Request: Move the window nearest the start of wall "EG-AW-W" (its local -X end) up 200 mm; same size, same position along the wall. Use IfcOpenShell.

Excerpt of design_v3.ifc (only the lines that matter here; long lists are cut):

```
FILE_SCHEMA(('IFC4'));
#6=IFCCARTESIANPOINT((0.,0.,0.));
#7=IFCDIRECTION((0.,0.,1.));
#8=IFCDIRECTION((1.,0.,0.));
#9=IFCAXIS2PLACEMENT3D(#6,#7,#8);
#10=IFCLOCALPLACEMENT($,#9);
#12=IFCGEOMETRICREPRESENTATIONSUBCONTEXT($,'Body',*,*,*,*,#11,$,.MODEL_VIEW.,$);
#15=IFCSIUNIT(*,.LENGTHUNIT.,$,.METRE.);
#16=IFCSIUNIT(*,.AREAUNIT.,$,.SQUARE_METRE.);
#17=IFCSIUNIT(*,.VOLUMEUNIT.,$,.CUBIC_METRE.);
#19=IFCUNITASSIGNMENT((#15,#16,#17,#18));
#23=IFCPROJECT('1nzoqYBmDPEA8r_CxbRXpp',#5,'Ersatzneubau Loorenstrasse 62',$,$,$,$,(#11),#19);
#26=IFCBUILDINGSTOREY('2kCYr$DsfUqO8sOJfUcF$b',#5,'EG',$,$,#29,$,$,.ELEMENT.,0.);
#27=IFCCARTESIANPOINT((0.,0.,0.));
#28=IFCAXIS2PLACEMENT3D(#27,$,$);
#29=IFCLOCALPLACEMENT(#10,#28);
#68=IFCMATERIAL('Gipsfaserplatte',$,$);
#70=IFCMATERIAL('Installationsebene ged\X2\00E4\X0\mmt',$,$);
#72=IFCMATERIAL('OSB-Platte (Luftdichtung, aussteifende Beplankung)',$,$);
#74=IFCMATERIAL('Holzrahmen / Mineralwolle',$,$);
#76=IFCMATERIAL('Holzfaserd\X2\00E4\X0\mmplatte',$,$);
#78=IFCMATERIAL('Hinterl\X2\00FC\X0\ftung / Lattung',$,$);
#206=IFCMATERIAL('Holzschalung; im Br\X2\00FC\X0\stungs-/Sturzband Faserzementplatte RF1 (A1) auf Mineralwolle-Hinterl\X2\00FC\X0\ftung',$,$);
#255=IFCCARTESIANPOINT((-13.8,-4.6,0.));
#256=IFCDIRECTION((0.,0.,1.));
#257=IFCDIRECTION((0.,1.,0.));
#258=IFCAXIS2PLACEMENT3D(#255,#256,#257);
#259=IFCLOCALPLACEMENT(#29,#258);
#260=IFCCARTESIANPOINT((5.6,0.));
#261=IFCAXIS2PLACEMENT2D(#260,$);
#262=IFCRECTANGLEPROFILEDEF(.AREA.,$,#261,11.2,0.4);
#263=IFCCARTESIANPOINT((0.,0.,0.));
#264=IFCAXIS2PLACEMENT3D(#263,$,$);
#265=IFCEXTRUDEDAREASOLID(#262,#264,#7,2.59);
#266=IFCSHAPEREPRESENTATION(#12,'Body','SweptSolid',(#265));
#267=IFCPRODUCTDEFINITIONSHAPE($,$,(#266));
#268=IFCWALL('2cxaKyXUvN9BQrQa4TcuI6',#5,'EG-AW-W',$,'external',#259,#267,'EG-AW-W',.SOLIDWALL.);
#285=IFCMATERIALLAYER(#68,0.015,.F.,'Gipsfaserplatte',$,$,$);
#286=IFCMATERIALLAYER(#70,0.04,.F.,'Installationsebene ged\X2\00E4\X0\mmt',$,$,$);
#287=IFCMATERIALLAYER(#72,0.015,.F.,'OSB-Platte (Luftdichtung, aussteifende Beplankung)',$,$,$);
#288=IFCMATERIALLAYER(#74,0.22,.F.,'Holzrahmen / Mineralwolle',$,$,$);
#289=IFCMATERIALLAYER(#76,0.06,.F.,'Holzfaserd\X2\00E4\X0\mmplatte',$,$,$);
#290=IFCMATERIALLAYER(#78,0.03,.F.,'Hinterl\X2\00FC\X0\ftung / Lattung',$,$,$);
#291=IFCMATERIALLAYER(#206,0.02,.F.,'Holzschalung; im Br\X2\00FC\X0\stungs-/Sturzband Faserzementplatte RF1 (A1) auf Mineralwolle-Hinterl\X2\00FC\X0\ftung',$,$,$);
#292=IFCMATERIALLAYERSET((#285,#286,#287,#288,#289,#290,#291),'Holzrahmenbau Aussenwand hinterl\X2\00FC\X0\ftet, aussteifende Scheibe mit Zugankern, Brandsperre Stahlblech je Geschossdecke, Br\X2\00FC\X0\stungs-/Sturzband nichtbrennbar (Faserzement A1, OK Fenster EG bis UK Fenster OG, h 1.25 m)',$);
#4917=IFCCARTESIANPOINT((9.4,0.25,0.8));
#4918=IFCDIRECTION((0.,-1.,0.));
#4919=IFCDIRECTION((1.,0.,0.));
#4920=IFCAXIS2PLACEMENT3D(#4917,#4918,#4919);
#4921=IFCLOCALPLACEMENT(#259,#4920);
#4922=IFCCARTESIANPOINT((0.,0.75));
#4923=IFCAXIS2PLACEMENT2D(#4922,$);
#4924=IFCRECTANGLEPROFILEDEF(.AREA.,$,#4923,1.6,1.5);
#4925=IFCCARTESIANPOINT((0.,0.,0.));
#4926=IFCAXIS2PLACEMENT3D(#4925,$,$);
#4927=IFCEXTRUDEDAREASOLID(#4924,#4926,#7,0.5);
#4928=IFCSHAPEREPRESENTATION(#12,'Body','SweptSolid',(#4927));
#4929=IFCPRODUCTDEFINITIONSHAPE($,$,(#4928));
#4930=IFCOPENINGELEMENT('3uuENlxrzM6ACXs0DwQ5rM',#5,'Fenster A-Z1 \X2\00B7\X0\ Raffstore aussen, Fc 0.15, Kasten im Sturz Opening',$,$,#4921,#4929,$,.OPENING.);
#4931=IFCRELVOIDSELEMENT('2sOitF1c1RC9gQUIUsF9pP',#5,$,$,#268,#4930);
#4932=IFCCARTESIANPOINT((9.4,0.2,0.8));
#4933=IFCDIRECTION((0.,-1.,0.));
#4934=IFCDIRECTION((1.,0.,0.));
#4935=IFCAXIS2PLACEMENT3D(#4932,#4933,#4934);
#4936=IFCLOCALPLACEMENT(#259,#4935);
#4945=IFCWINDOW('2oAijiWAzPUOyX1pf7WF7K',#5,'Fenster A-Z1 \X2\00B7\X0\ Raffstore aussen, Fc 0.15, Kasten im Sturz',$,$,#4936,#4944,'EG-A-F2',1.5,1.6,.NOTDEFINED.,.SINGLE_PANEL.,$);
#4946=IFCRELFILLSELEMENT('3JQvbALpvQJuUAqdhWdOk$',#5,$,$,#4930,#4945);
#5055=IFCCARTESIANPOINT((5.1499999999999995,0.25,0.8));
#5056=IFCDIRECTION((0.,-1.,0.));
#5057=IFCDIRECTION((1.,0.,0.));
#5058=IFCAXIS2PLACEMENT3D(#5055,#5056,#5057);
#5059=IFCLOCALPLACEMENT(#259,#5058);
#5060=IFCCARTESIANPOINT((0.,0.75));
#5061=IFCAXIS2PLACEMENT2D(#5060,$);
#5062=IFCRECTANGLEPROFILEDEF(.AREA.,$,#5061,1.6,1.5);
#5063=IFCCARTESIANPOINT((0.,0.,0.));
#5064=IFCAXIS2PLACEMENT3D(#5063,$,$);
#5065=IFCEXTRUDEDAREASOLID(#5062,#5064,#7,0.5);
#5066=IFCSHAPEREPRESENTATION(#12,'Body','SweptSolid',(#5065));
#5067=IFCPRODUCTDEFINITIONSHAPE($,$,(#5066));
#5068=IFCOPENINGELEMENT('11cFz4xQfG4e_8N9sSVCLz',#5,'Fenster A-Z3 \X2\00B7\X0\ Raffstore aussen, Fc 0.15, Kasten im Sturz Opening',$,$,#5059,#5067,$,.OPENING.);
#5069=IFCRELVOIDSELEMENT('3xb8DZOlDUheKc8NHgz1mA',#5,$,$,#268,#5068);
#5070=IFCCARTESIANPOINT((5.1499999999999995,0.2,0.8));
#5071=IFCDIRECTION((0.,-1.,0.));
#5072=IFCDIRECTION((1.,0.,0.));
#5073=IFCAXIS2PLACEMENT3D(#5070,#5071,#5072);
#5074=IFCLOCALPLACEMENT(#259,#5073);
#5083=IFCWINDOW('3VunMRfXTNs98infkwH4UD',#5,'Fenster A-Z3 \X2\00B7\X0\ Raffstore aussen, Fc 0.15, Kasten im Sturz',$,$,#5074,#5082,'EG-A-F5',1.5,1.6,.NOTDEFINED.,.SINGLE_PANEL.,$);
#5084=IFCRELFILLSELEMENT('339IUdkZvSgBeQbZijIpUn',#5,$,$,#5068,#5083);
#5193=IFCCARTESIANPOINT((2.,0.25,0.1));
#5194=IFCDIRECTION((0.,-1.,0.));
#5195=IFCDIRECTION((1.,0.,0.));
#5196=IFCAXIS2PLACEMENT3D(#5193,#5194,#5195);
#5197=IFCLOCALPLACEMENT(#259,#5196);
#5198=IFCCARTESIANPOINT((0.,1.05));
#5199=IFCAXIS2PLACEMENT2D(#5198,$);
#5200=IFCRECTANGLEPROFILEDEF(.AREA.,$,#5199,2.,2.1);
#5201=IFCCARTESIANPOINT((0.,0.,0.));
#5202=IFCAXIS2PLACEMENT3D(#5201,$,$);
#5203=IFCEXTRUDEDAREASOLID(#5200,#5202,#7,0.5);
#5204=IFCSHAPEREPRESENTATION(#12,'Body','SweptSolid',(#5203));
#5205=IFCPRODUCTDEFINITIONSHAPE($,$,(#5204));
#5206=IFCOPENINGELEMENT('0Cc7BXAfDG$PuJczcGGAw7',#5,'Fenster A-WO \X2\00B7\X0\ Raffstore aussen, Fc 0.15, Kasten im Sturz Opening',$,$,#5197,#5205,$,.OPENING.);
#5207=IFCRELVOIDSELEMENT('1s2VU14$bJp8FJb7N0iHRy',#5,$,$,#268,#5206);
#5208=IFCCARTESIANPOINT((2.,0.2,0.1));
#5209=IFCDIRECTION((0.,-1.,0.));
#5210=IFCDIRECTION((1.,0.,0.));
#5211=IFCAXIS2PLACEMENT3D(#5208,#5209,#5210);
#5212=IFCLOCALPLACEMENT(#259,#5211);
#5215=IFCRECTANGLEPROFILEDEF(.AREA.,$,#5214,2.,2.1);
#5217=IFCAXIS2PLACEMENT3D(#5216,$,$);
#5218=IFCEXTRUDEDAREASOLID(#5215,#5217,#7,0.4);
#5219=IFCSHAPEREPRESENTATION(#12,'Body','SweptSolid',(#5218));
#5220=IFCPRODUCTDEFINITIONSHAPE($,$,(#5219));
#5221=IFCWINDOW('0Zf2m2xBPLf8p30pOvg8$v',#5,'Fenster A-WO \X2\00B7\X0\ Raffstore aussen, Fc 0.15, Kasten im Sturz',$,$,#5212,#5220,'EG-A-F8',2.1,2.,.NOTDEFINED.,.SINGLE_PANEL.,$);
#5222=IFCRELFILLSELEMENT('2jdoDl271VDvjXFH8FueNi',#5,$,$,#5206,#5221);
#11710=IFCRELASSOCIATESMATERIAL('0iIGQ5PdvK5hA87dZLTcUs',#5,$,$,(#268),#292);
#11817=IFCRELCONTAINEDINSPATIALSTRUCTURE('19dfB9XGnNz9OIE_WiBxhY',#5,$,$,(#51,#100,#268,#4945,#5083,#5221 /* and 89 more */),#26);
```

```python
import numpy as np
import ifcopenshell
import ifcopenshell.api.geometry
import ifcopenshell.util.placement
import ifcopenshell.util.unit

model = ifcopenshell.open("design_v3.ifc")
unit_scale = ifcopenshell.util.unit.calculate_unit_scale(model)

window = model.by_guid("0Zf2m2xBPLf8p30pOvg8$v")
opening = window.FillsVoids[0].RelatingOpeningElement
dz = 0.2 / unit_scale

shift = np.array([0.0, 0.0, dz])
# The window is not placed relative to its opening, so move both.
for product in (opening, window):
    matrix = ifcopenshell.util.placement.get_local_placement(product.ObjectPlacement)
    matrix[:3, 3] += shift
    ifcopenshell.api.geometry.edit_object_placement(model, product=product, matrix=matrix, is_si=False)

print(f"moved by {dz * unit_scale:+.3f} m")

model.write("design_v3_edited.ifc")
```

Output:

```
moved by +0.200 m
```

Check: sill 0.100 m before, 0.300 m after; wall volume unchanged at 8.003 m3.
